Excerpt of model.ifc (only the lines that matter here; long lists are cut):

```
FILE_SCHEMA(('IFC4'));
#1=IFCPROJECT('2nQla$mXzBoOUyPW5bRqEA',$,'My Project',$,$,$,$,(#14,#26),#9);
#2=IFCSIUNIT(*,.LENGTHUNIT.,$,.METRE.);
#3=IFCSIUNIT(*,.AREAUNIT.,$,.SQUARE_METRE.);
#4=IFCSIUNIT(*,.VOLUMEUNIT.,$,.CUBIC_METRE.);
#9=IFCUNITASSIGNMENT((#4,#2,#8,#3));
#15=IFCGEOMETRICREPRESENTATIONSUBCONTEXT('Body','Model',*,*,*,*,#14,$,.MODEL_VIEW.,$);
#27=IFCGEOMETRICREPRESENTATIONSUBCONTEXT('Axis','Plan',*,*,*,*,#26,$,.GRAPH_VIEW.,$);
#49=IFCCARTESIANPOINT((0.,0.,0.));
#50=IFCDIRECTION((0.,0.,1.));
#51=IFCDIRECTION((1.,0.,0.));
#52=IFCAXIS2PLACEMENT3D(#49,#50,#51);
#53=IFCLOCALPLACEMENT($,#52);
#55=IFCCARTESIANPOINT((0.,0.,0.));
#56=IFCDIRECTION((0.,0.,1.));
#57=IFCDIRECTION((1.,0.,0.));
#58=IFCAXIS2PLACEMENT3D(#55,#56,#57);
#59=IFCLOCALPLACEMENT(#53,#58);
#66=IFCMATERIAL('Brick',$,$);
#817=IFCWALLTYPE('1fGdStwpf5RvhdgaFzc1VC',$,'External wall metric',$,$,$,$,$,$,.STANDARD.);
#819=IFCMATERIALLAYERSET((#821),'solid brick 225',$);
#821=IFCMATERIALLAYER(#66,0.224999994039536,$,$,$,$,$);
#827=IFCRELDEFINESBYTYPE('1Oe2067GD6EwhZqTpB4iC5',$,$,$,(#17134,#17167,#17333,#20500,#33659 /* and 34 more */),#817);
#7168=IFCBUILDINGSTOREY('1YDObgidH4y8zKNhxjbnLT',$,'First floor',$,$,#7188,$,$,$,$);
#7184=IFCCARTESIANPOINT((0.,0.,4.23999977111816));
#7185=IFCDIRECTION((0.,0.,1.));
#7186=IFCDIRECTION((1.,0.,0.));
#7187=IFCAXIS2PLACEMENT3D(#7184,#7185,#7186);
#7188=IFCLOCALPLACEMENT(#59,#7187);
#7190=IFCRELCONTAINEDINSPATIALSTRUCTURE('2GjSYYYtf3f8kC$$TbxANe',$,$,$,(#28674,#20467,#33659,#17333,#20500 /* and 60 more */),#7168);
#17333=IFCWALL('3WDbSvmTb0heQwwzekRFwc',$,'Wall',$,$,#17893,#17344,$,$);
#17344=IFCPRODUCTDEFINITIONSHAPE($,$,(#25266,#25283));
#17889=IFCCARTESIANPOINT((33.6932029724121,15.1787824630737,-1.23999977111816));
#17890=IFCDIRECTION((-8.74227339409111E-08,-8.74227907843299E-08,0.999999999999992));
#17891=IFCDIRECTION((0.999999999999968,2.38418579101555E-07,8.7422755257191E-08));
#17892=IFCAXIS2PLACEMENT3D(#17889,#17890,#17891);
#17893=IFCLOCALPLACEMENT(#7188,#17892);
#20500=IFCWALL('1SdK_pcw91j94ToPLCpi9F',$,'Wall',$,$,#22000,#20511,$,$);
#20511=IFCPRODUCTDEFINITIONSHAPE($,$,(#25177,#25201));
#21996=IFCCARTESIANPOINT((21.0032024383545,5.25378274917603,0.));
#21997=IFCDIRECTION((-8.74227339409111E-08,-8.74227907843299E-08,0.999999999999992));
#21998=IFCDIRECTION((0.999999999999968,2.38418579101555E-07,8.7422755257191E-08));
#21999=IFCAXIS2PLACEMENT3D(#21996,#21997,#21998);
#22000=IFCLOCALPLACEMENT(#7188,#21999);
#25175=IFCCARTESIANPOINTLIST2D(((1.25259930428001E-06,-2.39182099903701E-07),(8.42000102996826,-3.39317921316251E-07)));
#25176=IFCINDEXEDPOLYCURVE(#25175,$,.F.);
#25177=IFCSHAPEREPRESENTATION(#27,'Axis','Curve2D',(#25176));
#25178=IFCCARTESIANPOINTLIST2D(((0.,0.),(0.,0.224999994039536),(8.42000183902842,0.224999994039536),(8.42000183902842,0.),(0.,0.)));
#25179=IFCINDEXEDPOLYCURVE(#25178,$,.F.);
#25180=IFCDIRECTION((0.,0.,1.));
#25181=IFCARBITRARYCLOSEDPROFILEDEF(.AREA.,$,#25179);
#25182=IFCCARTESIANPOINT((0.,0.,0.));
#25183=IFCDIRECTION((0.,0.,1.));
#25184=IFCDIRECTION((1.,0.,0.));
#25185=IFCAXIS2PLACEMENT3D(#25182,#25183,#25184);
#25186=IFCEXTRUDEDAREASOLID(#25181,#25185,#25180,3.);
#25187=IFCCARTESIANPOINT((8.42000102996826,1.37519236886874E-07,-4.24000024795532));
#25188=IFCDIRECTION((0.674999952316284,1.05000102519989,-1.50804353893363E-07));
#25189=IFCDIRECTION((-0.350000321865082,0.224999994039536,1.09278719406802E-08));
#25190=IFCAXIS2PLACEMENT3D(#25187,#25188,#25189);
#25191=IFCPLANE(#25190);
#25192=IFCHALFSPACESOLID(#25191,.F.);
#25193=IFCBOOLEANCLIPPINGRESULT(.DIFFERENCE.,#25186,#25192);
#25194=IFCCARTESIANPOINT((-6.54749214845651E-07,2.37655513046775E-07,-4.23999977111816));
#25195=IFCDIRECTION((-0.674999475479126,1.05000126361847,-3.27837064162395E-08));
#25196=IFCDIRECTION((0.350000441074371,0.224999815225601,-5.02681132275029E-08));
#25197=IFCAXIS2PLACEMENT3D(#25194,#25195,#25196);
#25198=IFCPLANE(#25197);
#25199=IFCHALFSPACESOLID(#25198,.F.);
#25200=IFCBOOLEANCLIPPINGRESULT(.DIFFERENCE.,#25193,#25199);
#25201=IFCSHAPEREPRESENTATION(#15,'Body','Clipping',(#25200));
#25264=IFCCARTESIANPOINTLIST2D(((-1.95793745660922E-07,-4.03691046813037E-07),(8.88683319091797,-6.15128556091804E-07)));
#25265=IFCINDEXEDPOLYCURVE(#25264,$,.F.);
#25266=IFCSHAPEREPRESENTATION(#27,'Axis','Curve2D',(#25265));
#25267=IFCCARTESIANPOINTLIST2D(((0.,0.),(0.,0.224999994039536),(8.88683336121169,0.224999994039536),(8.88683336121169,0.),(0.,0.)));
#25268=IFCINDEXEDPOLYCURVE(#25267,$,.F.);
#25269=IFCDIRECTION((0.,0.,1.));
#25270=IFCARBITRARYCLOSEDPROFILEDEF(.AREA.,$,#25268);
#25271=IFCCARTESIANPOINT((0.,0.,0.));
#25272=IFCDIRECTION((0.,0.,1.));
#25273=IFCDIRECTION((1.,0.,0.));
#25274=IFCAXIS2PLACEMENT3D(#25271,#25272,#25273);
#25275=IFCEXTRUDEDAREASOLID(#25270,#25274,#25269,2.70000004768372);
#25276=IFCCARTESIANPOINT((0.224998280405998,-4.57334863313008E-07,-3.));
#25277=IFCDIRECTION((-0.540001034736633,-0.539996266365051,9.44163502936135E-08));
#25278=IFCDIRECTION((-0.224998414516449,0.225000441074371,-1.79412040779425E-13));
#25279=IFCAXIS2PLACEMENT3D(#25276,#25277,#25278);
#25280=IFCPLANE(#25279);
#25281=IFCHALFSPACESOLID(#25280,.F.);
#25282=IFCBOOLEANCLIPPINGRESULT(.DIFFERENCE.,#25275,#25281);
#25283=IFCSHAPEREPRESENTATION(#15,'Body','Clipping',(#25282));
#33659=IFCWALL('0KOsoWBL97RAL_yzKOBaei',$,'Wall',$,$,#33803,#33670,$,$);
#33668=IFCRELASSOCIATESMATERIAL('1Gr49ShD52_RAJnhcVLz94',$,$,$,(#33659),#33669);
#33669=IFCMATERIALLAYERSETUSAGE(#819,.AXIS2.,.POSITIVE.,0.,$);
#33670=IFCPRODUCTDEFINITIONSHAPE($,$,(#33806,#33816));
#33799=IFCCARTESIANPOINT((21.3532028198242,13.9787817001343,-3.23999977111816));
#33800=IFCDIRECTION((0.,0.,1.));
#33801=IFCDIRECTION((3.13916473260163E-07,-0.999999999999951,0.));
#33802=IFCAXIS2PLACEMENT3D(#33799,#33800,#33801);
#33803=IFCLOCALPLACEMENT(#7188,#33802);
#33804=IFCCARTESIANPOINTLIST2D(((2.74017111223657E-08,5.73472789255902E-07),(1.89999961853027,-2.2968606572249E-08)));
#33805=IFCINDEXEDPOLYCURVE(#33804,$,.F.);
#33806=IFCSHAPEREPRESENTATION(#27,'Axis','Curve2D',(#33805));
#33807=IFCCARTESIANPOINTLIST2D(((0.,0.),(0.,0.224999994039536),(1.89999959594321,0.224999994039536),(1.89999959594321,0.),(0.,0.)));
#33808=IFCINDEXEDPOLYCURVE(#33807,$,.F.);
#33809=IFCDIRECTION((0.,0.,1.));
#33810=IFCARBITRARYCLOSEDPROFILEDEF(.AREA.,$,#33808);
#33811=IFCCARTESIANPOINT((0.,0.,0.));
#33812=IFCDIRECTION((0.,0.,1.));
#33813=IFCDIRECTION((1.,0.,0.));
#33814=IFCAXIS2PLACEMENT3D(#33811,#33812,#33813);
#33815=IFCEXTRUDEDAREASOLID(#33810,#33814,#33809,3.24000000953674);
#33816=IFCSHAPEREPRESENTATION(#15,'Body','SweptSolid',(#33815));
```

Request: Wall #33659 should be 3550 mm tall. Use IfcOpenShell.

```python
import ifcopenshell
import ifcopenshell.geom
import ifcopenshell.util.representation
import ifcopenshell.util.shape

model = ifcopenshell.open("model.ifc")
settings = ifcopenshell.geom.settings()


def volume(element):
    """Net volume in cubic metres, openings subtracted."""
    shape = ifcopenshell.geom.create_shape(settings, element)
    return ifcopenshell.util.shape.get_volume(shape.geometry)


wall = model.by_guid("0KOsoWBL97RAL_yzKOBaei")
before = volume(wall)

body = ifcopenshell.util.representation.get_representation(wall, "Model", "Body")
solid = body.Items[0]
old_height = solid.Depth
solid.Depth = 3.55
after = volume(wall)

print(f"height {old_height:g} -> {solid.Depth:g}, volume {before:.3f} -> {after:.3f} m3")

model.write("model_edited.ifc")
```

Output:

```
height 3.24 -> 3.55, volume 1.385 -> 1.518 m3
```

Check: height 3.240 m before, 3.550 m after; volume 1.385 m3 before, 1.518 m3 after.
